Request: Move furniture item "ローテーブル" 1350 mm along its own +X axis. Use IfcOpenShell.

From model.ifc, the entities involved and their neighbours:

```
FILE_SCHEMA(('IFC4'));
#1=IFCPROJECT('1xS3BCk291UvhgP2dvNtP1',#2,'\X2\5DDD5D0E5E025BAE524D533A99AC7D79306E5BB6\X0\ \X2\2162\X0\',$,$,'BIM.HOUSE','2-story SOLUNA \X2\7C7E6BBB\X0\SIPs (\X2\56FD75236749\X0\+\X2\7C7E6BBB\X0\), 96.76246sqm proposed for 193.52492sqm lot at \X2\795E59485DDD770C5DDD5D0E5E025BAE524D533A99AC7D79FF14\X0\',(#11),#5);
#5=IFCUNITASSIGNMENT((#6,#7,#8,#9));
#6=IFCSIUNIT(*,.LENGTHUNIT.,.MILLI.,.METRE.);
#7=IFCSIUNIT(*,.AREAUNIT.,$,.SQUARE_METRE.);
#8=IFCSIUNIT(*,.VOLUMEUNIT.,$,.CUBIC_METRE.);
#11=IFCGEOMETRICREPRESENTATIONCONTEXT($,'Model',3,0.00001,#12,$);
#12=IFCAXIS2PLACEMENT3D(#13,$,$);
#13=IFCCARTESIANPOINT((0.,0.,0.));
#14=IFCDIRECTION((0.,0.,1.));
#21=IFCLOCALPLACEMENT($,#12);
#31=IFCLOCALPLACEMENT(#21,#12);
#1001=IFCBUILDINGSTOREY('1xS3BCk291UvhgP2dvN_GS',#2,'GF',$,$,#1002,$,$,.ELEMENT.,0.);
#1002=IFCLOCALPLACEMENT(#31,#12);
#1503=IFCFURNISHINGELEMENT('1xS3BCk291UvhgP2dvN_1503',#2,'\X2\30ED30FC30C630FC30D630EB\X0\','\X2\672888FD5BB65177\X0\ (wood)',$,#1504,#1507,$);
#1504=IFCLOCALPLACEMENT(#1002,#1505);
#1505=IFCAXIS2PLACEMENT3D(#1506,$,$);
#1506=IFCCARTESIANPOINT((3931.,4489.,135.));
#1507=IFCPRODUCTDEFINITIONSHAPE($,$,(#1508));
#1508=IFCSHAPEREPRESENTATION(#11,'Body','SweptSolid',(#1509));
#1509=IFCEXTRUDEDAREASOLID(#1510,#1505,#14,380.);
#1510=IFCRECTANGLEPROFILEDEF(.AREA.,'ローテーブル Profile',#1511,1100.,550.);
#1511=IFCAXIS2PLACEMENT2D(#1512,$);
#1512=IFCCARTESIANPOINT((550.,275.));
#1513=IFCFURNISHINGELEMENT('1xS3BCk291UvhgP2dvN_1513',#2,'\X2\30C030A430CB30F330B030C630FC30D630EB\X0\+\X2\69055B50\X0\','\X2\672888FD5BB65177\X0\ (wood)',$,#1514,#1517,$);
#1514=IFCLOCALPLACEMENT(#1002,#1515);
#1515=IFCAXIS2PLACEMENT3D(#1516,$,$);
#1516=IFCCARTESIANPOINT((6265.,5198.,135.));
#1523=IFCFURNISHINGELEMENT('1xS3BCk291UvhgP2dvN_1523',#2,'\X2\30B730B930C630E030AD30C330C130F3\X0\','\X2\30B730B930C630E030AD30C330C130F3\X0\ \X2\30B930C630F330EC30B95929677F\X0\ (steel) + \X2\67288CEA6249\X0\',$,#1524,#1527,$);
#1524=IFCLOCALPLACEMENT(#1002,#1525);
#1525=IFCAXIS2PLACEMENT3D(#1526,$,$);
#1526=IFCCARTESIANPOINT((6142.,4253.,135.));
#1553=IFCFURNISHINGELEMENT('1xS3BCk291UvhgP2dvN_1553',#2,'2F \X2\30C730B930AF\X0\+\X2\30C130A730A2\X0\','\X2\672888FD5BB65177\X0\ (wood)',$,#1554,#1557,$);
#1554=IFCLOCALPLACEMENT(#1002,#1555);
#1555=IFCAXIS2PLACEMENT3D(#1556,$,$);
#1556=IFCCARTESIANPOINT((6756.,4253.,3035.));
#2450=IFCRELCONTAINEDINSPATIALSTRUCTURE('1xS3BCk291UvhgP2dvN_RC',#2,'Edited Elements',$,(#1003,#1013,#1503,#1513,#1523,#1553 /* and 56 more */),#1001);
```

```python
import ifcopenshell
import ifcopenshell.api.geometry
import ifcopenshell.util.placement

model = ifcopenshell.open("model.ifc")

item = model.by_id(1503)
matrix = ifcopenshell.util.placement.get_local_placement(item.ObjectPlacement)
matrix[:3, 3] += matrix[:3, 0] * 1350.0
ifcopenshell.api.geometry.edit_object_placement(model, product=item, matrix=matrix, is_si=False)

print(ifcopenshell.util.placement.get_local_placement(item.ObjectPlacement).round(3) + 0.0)

model.write("model_updated.ifc")
```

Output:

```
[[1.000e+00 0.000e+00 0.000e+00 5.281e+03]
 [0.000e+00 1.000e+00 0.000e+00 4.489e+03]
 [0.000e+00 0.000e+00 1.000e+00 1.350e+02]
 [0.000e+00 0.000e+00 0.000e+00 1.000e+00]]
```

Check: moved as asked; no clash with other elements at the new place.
